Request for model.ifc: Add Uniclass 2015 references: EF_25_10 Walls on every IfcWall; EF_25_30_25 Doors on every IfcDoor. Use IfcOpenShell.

First a look at what the model holds.

```python
import ifcopenshell

model = ifcopenshell.open("model.ifc")
print(model.schema)
print("classifications:", [c.Name for c in model.by_type("IfcClassification")])
for ifc_class in ("IfcDoor", "IfcRoof", "IfcStair", "IfcWall", "IfcWindow"):
    print(ifc_class, len(model.by_type(ifc_class)))
```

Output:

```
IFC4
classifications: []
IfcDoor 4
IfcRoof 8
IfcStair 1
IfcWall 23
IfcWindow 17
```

```python
import ifcopenshell
import ifcopenshell.api.classification

model = ifcopenshell.open("model.ifc")

system = ifcopenshell.api.classification.add_classification(model, classification="Uniclass 2015")

codes = {
    "IfcWall": ("EF_25_10", "Walls"),
    "IfcDoor": ("EF_25_30_25", "Doors"),
}
for ifc_class, (code, name) in codes.items():
    products = model.by_type(ifc_class)
    ifcopenshell.api.classification.add_reference(
        model, products=products, classification=system, identification=code, name=name
    )
    print(code, len(products))

model.write("model-out.ifc")
```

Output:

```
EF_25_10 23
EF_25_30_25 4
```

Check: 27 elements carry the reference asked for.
